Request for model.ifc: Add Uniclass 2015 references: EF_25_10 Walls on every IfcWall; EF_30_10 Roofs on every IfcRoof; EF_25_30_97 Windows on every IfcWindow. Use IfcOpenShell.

First a look at what the model holds.

```python
import ifcopenshell

model = ifcopenshell.open("model.ifc")
print(model.schema)
print("classifications:", [c.Name for c in model.by_type("IfcClassification")])
for ifc_class in ("IfcDoor", "IfcRoof", "IfcStair", "IfcWall", "IfcWindow"):
    print(ifc_class, len(model.by_type(ifc_class)))
```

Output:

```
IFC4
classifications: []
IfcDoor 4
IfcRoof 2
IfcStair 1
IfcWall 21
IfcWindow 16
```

```python
import ifcopenshell
import ifcopenshell.api.classification

model = ifcopenshell.open("model.ifc")

system = ifcopenshell.api.classification.add_classification(model, classification="Uniclass 2015")

codes = {
    "IfcWall": ("EF_25_10", "Walls"),
    "IfcRoof": ("EF_30_10", "Roofs"),
    "IfcWindow": ("EF_25_30_97", "Windows"),
}
for ifc_class, (code, name) in codes.items():
    products = model.by_type(ifc_class)
    ifcopenshell.api.classification.add_reference(
        model, products=products, classification=system, identification=code, name=name
    )
    print(code, len(products))

model.write("model_v2.ifc")
```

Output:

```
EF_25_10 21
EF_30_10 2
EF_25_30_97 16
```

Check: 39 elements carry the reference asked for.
